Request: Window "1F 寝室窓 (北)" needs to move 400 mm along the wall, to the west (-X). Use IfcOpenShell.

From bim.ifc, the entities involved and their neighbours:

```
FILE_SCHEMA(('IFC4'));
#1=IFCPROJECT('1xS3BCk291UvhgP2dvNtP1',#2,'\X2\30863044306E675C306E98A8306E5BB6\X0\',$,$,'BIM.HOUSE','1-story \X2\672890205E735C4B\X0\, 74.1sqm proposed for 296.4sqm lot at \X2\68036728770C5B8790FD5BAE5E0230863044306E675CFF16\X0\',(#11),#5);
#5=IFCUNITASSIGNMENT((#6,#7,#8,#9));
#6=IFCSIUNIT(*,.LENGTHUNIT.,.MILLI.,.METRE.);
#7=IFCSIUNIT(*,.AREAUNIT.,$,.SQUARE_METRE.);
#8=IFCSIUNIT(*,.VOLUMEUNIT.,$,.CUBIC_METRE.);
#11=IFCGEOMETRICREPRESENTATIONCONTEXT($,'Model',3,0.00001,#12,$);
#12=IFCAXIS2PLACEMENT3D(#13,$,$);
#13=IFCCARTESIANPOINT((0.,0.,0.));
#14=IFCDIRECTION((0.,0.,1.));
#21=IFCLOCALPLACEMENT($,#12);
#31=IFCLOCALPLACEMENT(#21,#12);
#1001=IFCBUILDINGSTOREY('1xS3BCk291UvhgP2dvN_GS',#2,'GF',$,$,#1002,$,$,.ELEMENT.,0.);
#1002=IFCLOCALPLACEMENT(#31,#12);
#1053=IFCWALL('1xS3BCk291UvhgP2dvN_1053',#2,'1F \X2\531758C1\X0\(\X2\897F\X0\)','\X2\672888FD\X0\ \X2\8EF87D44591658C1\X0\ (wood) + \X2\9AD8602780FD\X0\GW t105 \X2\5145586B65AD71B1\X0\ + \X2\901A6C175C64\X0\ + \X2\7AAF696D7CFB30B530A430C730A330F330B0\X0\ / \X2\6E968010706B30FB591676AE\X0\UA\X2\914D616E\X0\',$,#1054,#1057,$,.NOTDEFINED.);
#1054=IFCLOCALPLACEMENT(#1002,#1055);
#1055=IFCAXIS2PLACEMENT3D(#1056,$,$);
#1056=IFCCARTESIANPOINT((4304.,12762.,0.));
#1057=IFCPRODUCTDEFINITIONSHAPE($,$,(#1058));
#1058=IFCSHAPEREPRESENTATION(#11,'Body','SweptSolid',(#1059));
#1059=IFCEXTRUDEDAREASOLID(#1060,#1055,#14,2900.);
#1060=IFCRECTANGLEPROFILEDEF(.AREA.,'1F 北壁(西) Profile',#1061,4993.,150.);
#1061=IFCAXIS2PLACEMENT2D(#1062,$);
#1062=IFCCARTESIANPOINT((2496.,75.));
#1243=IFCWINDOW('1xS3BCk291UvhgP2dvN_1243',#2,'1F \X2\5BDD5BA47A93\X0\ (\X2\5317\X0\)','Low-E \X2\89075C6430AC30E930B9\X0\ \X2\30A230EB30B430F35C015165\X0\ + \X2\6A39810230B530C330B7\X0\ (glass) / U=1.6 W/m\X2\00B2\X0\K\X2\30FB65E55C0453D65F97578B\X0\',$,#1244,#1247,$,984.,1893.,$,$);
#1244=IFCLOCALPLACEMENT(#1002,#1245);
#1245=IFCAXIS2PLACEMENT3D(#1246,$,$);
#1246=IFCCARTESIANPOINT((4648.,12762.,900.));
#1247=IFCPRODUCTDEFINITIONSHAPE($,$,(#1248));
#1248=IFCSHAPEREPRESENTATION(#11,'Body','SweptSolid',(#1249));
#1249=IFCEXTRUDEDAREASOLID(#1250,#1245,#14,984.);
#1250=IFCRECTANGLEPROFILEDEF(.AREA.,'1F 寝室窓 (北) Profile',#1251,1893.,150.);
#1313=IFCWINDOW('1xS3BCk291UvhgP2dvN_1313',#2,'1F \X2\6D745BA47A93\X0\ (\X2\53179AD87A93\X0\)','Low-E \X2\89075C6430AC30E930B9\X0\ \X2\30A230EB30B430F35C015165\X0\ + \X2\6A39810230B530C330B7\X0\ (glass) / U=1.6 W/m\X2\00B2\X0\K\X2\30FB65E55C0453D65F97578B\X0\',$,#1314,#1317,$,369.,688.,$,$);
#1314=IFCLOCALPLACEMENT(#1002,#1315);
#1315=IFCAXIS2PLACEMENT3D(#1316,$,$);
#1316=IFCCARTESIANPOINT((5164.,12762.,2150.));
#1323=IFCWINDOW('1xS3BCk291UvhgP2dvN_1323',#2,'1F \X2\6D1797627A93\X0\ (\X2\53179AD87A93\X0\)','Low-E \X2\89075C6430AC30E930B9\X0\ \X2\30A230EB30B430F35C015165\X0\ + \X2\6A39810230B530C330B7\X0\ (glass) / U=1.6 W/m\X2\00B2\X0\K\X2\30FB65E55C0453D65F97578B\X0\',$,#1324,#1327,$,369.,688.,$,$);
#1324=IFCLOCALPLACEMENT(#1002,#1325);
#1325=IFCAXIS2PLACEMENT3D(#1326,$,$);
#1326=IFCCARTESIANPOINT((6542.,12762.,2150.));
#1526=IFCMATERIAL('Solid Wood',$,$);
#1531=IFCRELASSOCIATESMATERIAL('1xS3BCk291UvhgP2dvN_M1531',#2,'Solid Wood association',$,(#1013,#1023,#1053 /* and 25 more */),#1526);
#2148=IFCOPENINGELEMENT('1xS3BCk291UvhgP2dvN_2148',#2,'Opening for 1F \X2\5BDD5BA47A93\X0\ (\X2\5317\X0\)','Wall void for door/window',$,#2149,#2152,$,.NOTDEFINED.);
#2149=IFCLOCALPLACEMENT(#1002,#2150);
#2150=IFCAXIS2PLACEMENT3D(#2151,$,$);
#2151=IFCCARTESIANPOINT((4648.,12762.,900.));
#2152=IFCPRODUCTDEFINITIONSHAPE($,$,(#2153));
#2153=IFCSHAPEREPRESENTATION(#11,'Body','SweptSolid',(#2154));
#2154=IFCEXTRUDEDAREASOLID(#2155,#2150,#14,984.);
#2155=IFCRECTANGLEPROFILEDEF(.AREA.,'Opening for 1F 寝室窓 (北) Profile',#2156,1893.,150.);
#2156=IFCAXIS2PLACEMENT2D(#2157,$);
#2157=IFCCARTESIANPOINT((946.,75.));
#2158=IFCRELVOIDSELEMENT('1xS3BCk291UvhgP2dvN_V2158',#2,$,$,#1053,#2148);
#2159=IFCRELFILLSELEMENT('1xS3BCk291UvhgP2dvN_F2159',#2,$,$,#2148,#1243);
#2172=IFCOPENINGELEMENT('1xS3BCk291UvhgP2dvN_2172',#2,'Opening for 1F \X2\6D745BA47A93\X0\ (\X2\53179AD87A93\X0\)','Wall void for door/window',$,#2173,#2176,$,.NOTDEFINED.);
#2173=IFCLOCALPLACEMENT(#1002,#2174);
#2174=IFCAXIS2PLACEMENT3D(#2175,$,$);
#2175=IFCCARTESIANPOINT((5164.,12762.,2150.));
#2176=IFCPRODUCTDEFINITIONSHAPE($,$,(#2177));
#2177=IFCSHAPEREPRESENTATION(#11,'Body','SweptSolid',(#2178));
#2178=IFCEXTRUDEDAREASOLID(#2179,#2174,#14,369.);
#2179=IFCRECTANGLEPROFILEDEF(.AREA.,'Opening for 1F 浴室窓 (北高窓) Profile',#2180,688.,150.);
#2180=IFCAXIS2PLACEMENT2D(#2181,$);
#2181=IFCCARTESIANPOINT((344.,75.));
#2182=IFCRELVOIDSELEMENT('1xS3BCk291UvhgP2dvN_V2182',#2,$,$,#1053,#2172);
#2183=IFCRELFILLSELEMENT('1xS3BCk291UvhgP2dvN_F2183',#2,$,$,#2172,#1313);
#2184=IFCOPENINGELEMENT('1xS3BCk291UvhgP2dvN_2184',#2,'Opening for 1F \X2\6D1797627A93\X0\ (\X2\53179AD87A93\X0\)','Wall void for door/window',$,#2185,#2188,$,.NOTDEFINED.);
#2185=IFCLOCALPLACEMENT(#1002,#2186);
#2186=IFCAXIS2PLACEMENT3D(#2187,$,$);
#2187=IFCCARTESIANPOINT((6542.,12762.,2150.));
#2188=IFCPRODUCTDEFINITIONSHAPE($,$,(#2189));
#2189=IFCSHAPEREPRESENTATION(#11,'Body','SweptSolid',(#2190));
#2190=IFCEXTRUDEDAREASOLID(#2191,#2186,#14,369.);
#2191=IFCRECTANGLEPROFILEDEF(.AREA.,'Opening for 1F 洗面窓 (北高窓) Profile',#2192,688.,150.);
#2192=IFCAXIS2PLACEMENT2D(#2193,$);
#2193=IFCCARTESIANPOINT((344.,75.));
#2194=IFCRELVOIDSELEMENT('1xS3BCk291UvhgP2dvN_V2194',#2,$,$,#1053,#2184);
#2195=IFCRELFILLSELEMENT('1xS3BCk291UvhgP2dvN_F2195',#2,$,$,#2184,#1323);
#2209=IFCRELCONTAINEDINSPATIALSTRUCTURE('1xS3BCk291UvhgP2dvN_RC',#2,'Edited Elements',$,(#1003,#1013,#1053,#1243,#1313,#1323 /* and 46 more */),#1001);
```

```python
import ifcopenshell
import ifcopenshell.api.geometry
import ifcopenshell.util.placement
import ifcopenshell.util.unit

model = ifcopenshell.open("bim.ifc")
unit_scale = ifcopenshell.util.unit.calculate_unit_scale(model)

window = model.by_id(1243)
opening = window.FillsVoids[0].RelatingOpeningElement
wall = opening.VoidsElements[0].RelatingBuildingElement

wall_matrix = ifcopenshell.util.placement.get_local_placement(wall.ObjectPlacement)
shift = wall_matrix[:3, 0] * -0.4 / unit_scale
before = ifcopenshell.util.placement.get_local_placement(window.ObjectPlacement)[:3, 3].copy()

# The window is not placed relative to its opening, so move both.
for product in (opening, window):
    matrix = ifcopenshell.util.placement.get_local_placement(product.ObjectPlacement)
    matrix[:3, 3] += shift
    ifcopenshell.api.geometry.edit_object_placement(model, product=product, matrix=matrix, is_si=False)

after = ifcopenshell.util.placement.get_local_placement(window.ObjectPlacement)[:3, 3]
print("window moved by", (after - before).round(3) + 0.0)

model.write("bim_rev.ifc")
```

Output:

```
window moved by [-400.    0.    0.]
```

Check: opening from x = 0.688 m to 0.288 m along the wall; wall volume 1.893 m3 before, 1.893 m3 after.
